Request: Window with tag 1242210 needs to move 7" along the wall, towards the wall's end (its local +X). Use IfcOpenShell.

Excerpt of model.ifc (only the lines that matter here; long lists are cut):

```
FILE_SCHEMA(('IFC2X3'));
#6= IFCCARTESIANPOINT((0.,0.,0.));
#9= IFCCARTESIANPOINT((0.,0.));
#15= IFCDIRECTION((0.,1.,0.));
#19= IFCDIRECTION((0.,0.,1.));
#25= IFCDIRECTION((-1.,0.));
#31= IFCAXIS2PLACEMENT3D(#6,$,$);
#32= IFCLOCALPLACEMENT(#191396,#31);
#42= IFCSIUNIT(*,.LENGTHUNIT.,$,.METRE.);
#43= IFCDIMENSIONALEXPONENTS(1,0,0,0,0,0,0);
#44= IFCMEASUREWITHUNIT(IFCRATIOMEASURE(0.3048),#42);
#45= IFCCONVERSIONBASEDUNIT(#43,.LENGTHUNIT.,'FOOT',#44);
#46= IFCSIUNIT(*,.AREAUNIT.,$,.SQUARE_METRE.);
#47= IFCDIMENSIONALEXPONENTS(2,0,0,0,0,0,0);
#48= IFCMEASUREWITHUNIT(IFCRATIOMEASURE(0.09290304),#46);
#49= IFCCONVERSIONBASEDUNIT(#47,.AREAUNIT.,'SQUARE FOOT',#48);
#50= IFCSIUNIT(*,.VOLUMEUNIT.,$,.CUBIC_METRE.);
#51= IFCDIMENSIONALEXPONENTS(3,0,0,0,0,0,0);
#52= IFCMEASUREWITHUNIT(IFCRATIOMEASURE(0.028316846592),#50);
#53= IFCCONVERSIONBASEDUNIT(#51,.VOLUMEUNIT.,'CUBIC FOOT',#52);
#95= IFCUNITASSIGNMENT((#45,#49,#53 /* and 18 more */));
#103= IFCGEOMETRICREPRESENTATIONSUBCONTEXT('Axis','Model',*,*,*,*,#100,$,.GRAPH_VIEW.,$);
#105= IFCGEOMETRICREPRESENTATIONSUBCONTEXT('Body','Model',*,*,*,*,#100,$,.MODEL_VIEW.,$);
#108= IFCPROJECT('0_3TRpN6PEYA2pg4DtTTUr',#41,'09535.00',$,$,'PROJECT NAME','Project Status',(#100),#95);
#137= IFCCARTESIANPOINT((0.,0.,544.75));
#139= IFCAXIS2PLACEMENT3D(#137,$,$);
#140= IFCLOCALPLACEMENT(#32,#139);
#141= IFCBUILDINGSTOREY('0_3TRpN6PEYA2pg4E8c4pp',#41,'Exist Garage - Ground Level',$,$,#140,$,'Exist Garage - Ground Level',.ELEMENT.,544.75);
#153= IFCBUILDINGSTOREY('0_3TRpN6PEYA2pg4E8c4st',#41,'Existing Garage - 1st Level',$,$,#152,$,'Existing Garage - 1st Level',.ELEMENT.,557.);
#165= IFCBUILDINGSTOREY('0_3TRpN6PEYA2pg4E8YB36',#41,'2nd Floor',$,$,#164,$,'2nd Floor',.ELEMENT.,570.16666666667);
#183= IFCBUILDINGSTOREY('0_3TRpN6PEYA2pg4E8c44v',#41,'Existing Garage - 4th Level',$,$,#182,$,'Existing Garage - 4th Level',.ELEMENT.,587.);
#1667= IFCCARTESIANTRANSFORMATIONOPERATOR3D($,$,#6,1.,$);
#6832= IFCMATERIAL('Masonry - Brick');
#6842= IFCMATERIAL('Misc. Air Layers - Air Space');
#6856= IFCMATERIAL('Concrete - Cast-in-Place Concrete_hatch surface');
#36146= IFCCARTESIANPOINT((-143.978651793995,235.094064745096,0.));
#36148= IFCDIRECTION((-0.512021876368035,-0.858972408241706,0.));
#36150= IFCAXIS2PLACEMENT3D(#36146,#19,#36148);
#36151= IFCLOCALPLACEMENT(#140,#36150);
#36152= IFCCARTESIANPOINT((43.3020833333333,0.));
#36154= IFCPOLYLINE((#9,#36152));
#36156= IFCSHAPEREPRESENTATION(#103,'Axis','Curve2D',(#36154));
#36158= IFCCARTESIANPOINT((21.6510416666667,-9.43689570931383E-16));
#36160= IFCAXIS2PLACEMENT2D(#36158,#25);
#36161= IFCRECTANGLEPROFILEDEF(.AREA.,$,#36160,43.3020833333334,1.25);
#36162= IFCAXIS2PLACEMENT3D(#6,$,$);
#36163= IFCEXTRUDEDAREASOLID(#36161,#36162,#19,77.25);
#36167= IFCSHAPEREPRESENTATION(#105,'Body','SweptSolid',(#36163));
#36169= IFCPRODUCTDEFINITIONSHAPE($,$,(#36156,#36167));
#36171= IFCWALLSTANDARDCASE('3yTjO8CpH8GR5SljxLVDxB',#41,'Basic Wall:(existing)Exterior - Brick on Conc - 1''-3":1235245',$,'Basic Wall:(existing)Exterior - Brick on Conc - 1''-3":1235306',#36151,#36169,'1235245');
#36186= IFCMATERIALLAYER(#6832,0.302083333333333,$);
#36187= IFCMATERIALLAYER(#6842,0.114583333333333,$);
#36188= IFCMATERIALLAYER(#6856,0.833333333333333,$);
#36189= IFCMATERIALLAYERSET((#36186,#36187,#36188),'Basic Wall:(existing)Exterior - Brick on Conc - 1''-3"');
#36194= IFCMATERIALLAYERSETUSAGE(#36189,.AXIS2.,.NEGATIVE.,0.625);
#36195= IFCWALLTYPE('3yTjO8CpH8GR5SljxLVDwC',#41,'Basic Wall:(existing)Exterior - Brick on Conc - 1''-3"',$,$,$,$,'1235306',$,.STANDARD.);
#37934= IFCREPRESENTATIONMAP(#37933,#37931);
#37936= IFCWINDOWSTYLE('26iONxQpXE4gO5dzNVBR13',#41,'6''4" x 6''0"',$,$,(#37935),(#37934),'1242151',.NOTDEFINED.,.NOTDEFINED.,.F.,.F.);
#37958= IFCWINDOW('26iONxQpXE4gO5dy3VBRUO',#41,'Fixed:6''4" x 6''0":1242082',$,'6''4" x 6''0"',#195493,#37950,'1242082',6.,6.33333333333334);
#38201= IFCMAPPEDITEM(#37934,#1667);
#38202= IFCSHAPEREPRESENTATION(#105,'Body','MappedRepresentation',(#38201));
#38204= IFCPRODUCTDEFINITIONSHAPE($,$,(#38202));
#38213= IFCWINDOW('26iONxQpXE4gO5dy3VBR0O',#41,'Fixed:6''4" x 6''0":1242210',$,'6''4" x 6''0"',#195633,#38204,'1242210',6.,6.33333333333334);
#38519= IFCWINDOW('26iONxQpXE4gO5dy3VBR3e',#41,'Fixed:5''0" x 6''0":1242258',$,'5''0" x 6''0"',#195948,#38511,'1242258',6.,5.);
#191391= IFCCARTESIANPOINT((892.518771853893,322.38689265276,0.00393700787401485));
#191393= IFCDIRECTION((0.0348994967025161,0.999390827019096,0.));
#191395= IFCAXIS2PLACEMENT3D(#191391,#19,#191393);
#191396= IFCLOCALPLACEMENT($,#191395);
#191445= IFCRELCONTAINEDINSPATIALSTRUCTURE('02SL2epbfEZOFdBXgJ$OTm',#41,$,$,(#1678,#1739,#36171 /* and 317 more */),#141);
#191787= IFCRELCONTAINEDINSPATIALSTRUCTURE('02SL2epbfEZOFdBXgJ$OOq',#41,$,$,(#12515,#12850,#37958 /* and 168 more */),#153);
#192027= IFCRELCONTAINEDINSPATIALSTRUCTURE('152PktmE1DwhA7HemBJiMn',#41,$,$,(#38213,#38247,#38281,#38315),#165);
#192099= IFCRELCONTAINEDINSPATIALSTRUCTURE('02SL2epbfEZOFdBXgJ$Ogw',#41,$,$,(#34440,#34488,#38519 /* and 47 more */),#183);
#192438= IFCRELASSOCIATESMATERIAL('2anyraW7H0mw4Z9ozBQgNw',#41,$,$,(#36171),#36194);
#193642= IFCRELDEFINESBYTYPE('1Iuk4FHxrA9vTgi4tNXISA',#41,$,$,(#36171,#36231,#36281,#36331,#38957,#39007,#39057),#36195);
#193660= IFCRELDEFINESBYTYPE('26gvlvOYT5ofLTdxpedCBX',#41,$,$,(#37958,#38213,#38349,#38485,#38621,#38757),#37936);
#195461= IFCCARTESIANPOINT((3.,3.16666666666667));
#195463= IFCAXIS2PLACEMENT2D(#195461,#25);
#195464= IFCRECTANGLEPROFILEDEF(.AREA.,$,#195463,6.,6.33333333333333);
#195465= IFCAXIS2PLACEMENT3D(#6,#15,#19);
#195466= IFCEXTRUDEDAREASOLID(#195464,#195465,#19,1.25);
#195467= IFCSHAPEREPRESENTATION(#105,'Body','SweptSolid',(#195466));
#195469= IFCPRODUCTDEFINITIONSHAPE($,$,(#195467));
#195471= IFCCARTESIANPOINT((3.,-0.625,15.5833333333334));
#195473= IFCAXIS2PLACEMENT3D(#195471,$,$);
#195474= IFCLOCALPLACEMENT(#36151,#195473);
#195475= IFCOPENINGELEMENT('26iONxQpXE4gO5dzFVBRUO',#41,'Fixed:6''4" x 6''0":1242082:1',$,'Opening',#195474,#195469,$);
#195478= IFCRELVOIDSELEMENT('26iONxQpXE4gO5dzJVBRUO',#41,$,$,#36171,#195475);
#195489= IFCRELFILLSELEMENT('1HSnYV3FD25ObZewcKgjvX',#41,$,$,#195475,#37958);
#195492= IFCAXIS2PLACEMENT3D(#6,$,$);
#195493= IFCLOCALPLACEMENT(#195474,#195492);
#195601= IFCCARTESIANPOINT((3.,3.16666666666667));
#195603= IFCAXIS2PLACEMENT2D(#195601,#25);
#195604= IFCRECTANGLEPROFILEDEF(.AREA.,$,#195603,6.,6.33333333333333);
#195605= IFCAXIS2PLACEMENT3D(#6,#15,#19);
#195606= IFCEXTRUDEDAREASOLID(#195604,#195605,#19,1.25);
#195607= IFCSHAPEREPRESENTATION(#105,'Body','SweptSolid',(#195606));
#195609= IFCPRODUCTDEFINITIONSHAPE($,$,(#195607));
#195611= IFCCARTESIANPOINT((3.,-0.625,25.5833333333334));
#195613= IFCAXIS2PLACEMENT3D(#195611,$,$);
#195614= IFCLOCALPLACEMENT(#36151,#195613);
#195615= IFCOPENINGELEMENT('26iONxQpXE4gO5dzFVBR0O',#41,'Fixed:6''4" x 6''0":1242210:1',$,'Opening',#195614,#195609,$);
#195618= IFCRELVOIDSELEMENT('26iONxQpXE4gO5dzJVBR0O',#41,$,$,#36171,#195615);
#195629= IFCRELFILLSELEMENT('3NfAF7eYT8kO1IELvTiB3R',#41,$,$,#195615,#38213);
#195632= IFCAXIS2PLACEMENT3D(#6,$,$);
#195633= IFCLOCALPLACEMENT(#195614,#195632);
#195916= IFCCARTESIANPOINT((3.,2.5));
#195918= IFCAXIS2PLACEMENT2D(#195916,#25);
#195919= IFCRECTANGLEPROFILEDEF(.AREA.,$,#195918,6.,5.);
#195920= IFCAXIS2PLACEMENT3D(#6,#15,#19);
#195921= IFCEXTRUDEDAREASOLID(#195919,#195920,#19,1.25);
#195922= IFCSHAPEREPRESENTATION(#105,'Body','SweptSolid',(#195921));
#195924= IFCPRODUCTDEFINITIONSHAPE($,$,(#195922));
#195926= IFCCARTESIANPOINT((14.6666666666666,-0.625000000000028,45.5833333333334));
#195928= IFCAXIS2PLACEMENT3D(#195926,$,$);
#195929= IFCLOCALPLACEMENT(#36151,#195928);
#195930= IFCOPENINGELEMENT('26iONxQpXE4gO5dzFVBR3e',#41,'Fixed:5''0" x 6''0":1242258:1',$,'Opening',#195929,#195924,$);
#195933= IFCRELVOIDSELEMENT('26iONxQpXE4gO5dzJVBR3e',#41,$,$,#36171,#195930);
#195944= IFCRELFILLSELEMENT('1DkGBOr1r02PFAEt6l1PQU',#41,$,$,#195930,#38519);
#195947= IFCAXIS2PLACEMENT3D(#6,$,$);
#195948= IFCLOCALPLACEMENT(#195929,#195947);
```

```python
import ifcopenshell
import ifcopenshell.api.geometry
import ifcopenshell.util.placement
import ifcopenshell.util.unit

model = ifcopenshell.open("model.ifc")
unit_scale = ifcopenshell.util.unit.calculate_unit_scale(model)

window = model.by_guid("26iONxQpXE4gO5dy3VBR0O")
opening = window.FillsVoids[0].RelatingOpeningElement
wall = opening.VoidsElements[0].RelatingBuildingElement

wall_matrix = ifcopenshell.util.placement.get_local_placement(wall.ObjectPlacement)
shift = wall_matrix[:3, 0] * 7 * 0.0254 / unit_scale
before = ifcopenshell.util.placement.get_local_placement(window.ObjectPlacement)[:3, 3].copy()

# The window is placed relative to its opening, so it follows when the opening moves.
matrix = ifcopenshell.util.placement.get_local_placement(opening.ObjectPlacement)
matrix[:3, 3] += shift
ifcopenshell.api.geometry.edit_object_placement(
    model, product=opening, matrix=matrix, is_si=False, should_transform_children=True
)

after = ifcopenshell.util.placement.get_local_placement(window.ObjectPlacement)[:3, 3]
print("window moved by", (after - before).round(3) + 0.0)

model.write("model_rev.ifc")
```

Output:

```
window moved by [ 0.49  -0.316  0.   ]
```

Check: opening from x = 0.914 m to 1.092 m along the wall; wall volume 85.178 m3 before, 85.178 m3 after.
